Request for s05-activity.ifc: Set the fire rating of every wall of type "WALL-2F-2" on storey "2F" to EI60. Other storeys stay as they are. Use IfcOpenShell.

First a look at what the model holds.

```python
import ifcopenshell
import ifcopenshell.util.element

model = ifcopenshell.open("s05-activity.ifc")
print(model.schema)
storey = next(s for s in model.by_type("IfcBuildingStorey") if s.Name == "2F")
walls = [e for e in ifcopenshell.util.element.get_decomposition(storey) if e.is_a("IfcWall")]
seen = {}
for e in walls:
    element_type = ifcopenshell.util.element.get_type(e)
    key = (element_type.Name if element_type != e and element_type else None, ifcopenshell.util.element.get_pset(e, "Pset_WallCommon", "FireRating"))
    seen[key] = seen.get(key, 0) + 1
for (name, value), count in sorted(seen.items(), key=str):
    print(count, "x", name, "|", value)
```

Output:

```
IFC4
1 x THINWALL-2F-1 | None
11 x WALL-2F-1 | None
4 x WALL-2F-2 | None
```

```python
import ifcopenshell
import ifcopenshell.api.pset
import ifcopenshell.util.element

model = ifcopenshell.open("s05-activity.ifc")

storey = next(s for s in model.by_type("IfcBuildingStorey") if s.Name == "2F")
walls = [e for e in ifcopenshell.util.element.get_decomposition(storey) if e.is_a("IfcWall")]

count = 0
for e in walls:
    element_type = ifcopenshell.util.element.get_type(e)
    if element_type in (None, e) or element_type.Name != "WALL-2F-2":
        continue
    # add_pset returns the element's existing set when there is one.
    pset = ifcopenshell.api.pset.add_pset(model, product=e, name="Pset_WallCommon")
    ifcopenshell.api.pset.edit_pset(model, pset=pset, properties={"FireRating": "EI60"})
    count += 1

print(count, "walls updated")

model.write("s05-activity_v2.ifc")
```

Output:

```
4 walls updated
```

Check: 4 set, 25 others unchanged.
